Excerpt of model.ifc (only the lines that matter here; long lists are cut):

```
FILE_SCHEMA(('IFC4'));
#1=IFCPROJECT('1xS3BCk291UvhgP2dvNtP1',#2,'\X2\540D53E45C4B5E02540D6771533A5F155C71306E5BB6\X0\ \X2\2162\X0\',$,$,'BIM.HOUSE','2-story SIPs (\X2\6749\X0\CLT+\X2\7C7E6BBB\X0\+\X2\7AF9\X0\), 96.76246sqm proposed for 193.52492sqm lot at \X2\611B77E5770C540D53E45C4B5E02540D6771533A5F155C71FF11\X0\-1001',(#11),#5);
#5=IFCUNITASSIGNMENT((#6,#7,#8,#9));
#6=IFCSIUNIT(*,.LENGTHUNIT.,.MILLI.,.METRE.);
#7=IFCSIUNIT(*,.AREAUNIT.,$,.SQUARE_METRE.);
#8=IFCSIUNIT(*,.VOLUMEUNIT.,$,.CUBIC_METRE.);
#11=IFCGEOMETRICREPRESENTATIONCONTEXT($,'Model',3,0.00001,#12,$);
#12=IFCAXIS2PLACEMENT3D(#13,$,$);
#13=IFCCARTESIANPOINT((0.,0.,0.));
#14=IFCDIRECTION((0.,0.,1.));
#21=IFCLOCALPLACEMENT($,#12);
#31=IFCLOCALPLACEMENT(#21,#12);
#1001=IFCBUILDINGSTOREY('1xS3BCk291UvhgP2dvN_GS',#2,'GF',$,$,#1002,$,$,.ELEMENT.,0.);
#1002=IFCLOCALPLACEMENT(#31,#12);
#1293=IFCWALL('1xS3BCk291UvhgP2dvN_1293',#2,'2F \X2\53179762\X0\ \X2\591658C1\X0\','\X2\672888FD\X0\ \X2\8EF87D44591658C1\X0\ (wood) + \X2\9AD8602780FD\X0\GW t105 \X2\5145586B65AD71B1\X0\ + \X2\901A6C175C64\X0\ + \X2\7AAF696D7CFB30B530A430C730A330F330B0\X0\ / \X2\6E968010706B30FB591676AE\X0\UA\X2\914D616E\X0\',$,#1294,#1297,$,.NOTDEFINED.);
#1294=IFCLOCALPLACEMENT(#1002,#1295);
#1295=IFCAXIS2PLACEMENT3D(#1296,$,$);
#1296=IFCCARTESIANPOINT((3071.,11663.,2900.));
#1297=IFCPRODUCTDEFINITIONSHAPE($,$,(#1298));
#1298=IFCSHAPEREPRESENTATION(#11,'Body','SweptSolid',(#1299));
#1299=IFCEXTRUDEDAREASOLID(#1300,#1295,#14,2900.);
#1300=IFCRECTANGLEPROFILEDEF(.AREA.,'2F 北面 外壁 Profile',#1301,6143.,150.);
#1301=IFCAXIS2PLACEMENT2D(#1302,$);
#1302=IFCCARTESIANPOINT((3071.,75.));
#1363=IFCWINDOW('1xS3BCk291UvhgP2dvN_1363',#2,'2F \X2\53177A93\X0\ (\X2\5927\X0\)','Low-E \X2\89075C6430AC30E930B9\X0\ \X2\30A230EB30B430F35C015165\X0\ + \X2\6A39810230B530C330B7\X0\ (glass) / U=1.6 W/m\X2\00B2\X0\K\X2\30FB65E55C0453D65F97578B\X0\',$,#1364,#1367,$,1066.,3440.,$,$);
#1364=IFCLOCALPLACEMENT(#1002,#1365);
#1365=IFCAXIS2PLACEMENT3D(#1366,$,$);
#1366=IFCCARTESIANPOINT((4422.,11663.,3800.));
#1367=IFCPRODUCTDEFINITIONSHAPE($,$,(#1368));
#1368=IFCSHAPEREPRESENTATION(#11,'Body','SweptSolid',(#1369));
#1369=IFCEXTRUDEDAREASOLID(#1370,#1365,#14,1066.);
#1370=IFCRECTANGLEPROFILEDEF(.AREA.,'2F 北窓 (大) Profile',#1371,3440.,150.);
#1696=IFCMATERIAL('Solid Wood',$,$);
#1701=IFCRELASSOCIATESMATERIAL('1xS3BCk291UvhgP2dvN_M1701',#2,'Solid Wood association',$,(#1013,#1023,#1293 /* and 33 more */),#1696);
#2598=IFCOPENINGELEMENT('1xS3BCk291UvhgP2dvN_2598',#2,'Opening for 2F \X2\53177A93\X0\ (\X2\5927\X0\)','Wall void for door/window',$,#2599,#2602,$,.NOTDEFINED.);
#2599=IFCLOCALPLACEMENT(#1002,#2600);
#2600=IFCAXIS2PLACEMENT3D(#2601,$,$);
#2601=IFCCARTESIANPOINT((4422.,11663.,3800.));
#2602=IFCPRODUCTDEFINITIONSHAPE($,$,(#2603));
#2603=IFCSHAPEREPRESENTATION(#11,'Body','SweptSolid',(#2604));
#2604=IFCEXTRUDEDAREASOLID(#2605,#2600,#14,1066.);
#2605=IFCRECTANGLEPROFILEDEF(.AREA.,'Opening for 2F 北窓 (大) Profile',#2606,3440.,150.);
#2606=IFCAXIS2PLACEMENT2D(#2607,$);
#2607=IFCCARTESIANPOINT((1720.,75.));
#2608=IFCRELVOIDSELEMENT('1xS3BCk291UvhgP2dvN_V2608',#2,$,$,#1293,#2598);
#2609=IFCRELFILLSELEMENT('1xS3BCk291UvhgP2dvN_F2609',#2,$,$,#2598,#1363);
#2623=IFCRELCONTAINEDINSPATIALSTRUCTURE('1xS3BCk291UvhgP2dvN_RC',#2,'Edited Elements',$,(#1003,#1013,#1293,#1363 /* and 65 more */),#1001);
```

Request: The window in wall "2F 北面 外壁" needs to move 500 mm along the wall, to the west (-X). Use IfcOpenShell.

```python
import ifcopenshell
import ifcopenshell.api.geometry
import ifcopenshell.util.placement
import ifcopenshell.util.unit

model = ifcopenshell.open("model.ifc")
unit_scale = ifcopenshell.util.unit.calculate_unit_scale(model)

window = model.by_id(1363)
opening = window.FillsVoids[0].RelatingOpeningElement
wall = opening.VoidsElements[0].RelatingBuildingElement

wall_matrix = ifcopenshell.util.placement.get_local_placement(wall.ObjectPlacement)
shift = wall_matrix[:3, 0] * -0.5 / unit_scale
before = ifcopenshell.util.placement.get_local_placement(window.ObjectPlacement)[:3, 3].copy()

# The window is not placed relative to its opening, so move both.
for product in (opening, window):
    matrix = ifcopenshell.util.placement.get_local_placement(product.ObjectPlacement)
    matrix[:3, 3] += shift
    ifcopenshell.api.geometry.edit_object_placement(model, product=product, matrix=matrix, is_si=False)

after = ifcopenshell.util.placement.get_local_placement(window.ObjectPlacement)[:3, 3]
print("window moved by", (after - before).round(3) + 0.0)

model.write("model_rev.ifc")
```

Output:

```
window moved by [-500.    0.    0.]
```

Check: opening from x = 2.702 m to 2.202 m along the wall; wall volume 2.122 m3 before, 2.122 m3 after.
